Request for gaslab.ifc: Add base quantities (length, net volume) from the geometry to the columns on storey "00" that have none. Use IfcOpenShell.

First a look at what the model holds.

```python
import ifcopenshell
import ifcopenshell.util.element
import ifcopenshell.util.unit

model = ifcopenshell.open("gaslab.ifc")
print(model.schema)
for unit_type in ("LENGTHUNIT", "AREAUNIT", "VOLUMEUNIT"):
    print(unit_type, ifcopenshell.util.unit.calculate_unit_scale(model, unit_type))
storey = next(s for s in model.by_type("IfcBuildingStorey") if s.Name == "00")
columns = [e for e in ifcopenshell.util.element.get_decomposition(storey) if e.is_a("IfcColumn")]
for e in sorted(columns, key=lambda e: e.id()):
    print(e.id(), e.is_a(), e.Name, list(ifcopenshell.util.element.get_psets(e, qtos_only=True)), sep=" | ")
```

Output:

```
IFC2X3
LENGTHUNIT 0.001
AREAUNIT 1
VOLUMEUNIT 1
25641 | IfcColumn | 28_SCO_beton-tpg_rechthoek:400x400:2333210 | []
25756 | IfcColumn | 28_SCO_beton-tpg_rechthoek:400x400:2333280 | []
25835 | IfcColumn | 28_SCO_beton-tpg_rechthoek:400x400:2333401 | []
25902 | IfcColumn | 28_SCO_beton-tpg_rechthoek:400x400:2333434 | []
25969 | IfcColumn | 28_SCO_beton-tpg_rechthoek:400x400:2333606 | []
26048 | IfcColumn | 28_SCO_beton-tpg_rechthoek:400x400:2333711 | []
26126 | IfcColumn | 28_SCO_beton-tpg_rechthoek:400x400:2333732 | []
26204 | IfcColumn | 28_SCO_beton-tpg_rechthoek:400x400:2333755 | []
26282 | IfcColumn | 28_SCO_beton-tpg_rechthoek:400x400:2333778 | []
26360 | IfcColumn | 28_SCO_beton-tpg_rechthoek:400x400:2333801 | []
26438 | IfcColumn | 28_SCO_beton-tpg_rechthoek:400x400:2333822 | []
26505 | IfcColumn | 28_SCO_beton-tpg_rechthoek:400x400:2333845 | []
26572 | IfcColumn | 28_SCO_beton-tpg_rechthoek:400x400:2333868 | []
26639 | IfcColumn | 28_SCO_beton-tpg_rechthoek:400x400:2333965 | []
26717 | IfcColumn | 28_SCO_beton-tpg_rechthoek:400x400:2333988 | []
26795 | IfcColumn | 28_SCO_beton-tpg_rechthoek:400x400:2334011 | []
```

```python
import ifcopenshell
import ifcopenshell.api.pset
import ifcopenshell.geom
import ifcopenshell.util.element
import ifcopenshell.util.shape
import ifcopenshell.util.unit

model = ifcopenshell.open("gaslab.ifc")
unit_scale = ifcopenshell.util.unit.calculate_unit_scale(model)
volume_scale = ifcopenshell.util.unit.calculate_unit_scale(model, "VOLUMEUNIT")
settings = ifcopenshell.geom.settings()

storey = next(s for s in model.by_type("IfcBuildingStorey") if s.Name == "00")
columns = [e for e in ifcopenshell.util.element.get_decomposition(storey) if e.is_a("IfcColumn")]

for e in sorted(columns, key=lambda e: e.id()):
    if ifcopenshell.util.element.get_psets(e, qtos_only=True, should_inherit=False):
        continue
    # Geometry comes back in metres, in the element's own axes.
    shape = ifcopenshell.geom.create_shape(settings, e)
    values = {
        "Length": ifcopenshell.util.shape.get_z(shape.geometry) / unit_scale,
        "NetVolume": ifcopenshell.util.shape.get_volume(shape.geometry) / volume_scale,
    }
    qto = ifcopenshell.api.pset.add_qto(model, product=e, name="BaseQuantities")
    ifcopenshell.api.pset.edit_qto(model, qto=qto, properties=values)
    print(e.id(), {k: round(v, 3) for k, v in values.items()})

model.write("gaslab_rev.ifc")
```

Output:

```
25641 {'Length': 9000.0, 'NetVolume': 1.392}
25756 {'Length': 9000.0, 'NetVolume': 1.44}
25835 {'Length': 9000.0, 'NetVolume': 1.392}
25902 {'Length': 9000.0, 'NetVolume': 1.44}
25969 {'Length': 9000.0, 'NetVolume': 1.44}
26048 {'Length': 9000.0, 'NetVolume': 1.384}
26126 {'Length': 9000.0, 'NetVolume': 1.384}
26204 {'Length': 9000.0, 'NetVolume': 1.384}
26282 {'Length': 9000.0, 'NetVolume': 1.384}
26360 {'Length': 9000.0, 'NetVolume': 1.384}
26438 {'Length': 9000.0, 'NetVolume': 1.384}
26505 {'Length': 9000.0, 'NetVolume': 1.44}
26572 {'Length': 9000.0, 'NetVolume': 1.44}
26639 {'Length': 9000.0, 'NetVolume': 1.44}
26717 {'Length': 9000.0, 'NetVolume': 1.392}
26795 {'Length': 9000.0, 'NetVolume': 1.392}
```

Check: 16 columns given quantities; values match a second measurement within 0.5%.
